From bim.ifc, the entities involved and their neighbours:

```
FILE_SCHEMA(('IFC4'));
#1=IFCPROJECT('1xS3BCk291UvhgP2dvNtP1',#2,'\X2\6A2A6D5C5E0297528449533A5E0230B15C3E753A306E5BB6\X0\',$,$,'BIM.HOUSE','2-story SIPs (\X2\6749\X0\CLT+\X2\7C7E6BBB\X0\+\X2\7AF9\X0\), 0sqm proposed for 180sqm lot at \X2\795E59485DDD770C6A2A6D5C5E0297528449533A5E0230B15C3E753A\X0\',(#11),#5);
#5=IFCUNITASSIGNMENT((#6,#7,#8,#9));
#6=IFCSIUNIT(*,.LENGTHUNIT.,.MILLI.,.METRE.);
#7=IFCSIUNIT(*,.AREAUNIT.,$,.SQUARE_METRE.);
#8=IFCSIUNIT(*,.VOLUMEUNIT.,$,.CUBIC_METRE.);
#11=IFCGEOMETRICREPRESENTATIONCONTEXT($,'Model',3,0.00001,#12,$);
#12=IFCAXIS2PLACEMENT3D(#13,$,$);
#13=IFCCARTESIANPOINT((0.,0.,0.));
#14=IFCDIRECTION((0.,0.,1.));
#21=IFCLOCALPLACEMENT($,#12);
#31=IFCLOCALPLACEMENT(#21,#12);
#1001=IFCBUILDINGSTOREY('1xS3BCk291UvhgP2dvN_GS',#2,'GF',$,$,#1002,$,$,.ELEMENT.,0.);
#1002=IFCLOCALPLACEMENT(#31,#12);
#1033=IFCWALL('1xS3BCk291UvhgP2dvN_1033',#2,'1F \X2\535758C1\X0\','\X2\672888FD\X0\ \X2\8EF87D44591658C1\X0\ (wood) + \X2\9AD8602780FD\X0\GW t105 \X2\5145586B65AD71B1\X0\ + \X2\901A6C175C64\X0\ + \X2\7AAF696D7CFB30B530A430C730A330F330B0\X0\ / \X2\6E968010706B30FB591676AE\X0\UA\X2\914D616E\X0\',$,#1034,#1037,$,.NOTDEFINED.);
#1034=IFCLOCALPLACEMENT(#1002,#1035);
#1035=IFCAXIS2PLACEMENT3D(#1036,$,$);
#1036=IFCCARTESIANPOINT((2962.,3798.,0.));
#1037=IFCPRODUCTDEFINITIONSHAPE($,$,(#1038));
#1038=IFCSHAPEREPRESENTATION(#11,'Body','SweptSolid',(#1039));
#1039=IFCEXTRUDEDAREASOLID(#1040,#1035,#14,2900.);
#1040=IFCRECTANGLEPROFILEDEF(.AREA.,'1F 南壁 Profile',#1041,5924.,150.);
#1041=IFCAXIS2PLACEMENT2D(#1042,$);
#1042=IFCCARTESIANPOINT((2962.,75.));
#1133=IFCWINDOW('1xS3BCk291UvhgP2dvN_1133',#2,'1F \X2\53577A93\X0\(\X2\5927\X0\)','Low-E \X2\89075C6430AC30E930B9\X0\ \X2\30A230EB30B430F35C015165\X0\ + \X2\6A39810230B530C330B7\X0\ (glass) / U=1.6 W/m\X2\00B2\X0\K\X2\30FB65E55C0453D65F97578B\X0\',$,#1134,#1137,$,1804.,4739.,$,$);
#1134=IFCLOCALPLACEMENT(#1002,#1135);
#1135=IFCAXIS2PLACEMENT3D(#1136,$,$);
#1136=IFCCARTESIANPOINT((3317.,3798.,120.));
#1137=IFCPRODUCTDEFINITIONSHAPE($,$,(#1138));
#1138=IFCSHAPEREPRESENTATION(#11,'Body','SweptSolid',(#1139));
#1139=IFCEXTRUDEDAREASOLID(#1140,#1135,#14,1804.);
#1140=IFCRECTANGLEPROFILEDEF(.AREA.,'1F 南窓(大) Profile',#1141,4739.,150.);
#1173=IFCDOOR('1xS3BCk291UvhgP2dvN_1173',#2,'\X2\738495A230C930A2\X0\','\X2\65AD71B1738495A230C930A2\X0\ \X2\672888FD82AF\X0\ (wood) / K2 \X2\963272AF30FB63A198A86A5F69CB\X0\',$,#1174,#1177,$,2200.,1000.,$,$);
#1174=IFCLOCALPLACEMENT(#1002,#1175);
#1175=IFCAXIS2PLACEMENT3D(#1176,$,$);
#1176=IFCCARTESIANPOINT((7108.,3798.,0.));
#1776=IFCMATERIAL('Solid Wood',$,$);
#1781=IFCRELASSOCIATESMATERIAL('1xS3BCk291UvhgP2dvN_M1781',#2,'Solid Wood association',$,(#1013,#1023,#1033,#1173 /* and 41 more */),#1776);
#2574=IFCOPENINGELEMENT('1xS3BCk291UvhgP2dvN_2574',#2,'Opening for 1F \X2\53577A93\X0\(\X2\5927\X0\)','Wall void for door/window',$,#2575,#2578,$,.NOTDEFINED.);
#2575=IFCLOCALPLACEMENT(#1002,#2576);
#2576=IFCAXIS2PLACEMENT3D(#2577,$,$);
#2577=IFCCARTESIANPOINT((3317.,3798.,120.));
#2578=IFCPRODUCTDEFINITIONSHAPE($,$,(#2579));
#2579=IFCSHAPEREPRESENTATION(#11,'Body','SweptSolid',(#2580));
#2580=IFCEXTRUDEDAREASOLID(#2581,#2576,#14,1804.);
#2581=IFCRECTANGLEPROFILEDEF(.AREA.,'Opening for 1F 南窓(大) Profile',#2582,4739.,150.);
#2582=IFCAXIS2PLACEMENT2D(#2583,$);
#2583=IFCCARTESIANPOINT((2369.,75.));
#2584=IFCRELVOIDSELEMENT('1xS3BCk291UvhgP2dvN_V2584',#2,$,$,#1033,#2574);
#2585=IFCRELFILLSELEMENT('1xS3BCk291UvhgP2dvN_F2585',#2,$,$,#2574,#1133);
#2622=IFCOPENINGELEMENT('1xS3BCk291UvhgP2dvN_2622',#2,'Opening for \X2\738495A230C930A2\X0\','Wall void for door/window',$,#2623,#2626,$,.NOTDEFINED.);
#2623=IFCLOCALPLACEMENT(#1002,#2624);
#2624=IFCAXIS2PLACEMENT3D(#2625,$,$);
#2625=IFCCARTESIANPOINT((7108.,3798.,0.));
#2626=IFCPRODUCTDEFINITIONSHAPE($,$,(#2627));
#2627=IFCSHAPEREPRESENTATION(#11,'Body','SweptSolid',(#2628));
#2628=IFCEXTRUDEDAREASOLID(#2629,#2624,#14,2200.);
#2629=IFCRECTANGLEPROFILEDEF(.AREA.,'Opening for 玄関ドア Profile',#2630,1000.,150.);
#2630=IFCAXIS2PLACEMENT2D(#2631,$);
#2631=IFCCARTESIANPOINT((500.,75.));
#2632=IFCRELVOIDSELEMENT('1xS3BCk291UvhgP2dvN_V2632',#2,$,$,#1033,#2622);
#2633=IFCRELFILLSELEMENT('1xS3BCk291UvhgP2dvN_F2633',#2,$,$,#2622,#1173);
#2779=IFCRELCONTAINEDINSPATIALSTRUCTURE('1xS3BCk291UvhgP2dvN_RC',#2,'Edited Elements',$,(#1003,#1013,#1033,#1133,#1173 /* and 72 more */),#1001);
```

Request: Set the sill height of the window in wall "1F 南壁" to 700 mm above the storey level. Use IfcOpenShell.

```python
import numpy as np
import ifcopenshell
import ifcopenshell.api.geometry
import ifcopenshell.geom
import ifcopenshell.util.element
import ifcopenshell.util.placement
import ifcopenshell.util.shape
import ifcopenshell.util.unit

model = ifcopenshell.open("bim.ifc")
unit_scale = ifcopenshell.util.unit.calculate_unit_scale(model)

window = model.by_id(1133)
opening = window.FillsVoids[0].RelatingOpeningElement
storey = ifcopenshell.util.element.get_container(window, ifc_class="IfcBuildingStorey")
level = ifcopenshell.util.placement.get_local_placement(storey.ObjectPlacement)[2, 3]

# The opening's origin need not be at the sill, so measure its lowest point.
shape = ifcopenshell.geom.create_shape(ifcopenshell.geom.settings(), opening)
bottom = ifcopenshell.util.shape.get_shape_bottom_elevation(shape, shape.geometry) / unit_scale
dz = level + 0.7 / unit_scale - bottom

shift = np.array([0.0, 0.0, dz])
# The window is not placed relative to its opening, so move both.
for product in (opening, window):
    matrix = ifcopenshell.util.placement.get_local_placement(product.ObjectPlacement)
    matrix[:3, 3] += shift
    ifcopenshell.api.geometry.edit_object_placement(model, product=product, matrix=matrix, is_si=False)

print(f"moved by {dz * unit_scale:+.3f} m")

model.write("bim_v2.ifc")
```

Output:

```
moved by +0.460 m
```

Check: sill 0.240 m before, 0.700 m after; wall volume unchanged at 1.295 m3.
